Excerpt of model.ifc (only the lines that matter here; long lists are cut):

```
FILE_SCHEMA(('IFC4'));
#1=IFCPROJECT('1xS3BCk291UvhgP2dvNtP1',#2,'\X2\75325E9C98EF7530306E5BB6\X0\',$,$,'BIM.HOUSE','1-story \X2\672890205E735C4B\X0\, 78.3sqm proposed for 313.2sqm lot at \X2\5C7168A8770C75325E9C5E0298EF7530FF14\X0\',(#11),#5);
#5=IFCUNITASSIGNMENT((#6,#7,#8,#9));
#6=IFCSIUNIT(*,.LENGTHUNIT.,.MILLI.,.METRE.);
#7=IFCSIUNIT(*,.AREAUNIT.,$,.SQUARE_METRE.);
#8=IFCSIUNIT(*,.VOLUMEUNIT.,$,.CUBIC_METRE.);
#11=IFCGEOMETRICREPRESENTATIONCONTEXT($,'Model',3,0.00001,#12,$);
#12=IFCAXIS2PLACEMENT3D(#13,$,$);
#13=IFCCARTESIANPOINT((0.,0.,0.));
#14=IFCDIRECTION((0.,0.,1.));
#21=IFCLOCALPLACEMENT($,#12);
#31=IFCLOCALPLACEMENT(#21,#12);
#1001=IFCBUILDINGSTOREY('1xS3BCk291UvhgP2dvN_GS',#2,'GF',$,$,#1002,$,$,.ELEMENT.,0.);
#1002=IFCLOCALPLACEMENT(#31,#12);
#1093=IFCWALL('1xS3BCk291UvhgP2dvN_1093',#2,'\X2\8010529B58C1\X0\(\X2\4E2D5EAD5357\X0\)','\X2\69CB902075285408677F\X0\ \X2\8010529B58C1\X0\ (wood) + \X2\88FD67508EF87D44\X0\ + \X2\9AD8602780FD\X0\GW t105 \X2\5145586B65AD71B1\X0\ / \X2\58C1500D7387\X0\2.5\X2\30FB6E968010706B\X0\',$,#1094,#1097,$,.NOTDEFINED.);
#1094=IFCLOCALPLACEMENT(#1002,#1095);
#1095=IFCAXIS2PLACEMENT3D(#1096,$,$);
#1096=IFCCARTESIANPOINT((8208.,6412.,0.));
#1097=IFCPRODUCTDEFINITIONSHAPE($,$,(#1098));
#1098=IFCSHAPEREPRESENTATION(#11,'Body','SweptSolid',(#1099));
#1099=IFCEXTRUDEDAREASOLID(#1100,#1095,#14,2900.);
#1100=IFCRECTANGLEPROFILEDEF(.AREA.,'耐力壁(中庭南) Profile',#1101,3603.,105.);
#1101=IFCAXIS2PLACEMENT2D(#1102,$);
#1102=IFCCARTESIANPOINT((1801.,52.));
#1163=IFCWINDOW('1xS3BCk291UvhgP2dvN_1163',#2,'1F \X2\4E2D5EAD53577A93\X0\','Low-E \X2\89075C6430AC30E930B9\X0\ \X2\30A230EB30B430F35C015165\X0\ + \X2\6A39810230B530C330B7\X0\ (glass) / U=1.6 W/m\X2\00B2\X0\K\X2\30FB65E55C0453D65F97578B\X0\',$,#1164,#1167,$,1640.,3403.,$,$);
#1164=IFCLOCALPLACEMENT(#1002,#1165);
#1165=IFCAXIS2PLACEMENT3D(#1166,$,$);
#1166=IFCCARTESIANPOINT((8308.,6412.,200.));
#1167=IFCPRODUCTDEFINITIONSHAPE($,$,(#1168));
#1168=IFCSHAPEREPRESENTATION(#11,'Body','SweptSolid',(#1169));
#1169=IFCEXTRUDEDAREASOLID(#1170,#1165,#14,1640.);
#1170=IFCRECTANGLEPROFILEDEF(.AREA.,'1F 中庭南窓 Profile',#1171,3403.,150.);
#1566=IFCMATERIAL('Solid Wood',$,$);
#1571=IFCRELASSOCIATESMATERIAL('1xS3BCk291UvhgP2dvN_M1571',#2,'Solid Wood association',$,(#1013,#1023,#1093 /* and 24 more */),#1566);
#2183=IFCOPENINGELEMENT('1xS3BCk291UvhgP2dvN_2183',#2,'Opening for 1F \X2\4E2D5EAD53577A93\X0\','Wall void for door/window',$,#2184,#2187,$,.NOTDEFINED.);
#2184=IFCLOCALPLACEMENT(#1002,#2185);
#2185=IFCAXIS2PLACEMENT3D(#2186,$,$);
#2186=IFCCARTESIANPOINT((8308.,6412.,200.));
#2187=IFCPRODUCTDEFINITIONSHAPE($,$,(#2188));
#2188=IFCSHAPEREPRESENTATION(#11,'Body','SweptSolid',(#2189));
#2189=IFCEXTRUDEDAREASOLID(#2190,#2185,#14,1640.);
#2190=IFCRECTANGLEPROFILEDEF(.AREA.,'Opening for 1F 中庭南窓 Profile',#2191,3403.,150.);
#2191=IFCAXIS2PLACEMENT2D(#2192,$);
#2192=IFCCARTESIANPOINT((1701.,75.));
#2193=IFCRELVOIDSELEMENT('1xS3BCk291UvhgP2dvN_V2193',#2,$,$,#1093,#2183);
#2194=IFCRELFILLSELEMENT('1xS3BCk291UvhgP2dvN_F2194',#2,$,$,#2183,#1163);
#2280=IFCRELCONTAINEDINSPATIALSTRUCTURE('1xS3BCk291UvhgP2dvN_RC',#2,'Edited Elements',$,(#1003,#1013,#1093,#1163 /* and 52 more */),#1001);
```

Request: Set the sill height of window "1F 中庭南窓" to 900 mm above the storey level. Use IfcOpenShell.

```python
import numpy as np
import ifcopenshell
import ifcopenshell.api.geometry
import ifcopenshell.geom
import ifcopenshell.util.element
import ifcopenshell.util.placement
import ifcopenshell.util.shape
import ifcopenshell.util.unit

model = ifcopenshell.open("model.ifc")
unit_scale = ifcopenshell.util.unit.calculate_unit_scale(model)

window = model.by_guid("1xS3BCk291UvhgP2dvN_1163")
opening = window.FillsVoids[0].RelatingOpeningElement
storey = ifcopenshell.util.element.get_container(window, ifc_class="IfcBuildingStorey")
level = ifcopenshell.util.placement.get_local_placement(storey.ObjectPlacement)[2, 3]

# The opening's origin need not be at the sill, so measure its lowest point.
shape = ifcopenshell.geom.create_shape(ifcopenshell.geom.settings(), opening)
bottom = ifcopenshell.util.shape.get_shape_bottom_elevation(shape, shape.geometry) / unit_scale
dz = level + 0.9 / unit_scale - bottom

shift = np.array([0.0, 0.0, dz])
# The window is not placed relative to its opening, so move both.
for product in (opening, window):
    matrix = ifcopenshell.util.placement.get_local_placement(product.ObjectPlacement)
    matrix[:3, 3] += shift
    ifcopenshell.api.geometry.edit_object_placement(model, product=product, matrix=matrix, is_si=False)

print(f"moved by {dz * unit_scale:+.3f} m")

model.write("model_updated.ifc")
```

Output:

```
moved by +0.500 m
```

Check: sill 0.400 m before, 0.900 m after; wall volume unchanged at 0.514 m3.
